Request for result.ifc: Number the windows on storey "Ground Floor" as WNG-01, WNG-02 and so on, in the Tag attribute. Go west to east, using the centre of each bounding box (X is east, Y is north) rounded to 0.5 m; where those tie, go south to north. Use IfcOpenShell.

First a look at what the model holds.

```python
import ifcopenshell
import ifcopenshell.util.element
import ifcopenshell.util.placement

model = ifcopenshell.open("result.ifc")
print(model.schema)
storey = next(s for s in model.by_type("IfcBuildingStorey") if s.Name == "Ground Floor")
windows = [e for e in ifcopenshell.util.element.get_decomposition(storey) if e.is_a("IfcWindow")]
for e in sorted(windows, key=lambda e: e.id()):
    origin = ifcopenshell.util.placement.get_local_placement(e.ObjectPlacement)[:3, 3]
    print(e.id(), e.Tag, e.Name, origin.round(2) + 0.0, sep=" | ")
```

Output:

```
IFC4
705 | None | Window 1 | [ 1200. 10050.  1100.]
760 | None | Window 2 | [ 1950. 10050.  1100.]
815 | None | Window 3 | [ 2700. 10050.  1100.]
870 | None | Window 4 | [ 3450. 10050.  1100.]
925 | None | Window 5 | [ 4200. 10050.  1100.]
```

```python
import ifcopenshell
import ifcopenshell.geom
import ifcopenshell.util.element
import ifcopenshell.util.shape

model = ifcopenshell.open("result.ifc")
settings = ifcopenshell.geom.settings()
settings.set("use-world-coords", True)


def centre(element):
    shape = ifcopenshell.geom.create_shape(settings, element)
    return ifcopenshell.util.shape.get_bbox_centroid(shape.geometry)


storey = next(s for s in model.by_type("IfcBuildingStorey") if s.Name == "Ground Floor")
windows = [e for e in ifcopenshell.util.element.get_decomposition(storey) if e.is_a("IfcWindow")]

# Insertion points can sit at a corner or the storey origin, so sort by the geometry (in metres).
centres = {e: centre(e) for e in windows}
windows.sort(key=lambda e: (round(centres[e][0] / 0.5), centres[e][1]))

for i, e in enumerate(windows, start=1):
    number = f"WNG-{i:02d}"
    e.Tag = number
    print(e.id(), number)

model.write("result_v2.ifc")
```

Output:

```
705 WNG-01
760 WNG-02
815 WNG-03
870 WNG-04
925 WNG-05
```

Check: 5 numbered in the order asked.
